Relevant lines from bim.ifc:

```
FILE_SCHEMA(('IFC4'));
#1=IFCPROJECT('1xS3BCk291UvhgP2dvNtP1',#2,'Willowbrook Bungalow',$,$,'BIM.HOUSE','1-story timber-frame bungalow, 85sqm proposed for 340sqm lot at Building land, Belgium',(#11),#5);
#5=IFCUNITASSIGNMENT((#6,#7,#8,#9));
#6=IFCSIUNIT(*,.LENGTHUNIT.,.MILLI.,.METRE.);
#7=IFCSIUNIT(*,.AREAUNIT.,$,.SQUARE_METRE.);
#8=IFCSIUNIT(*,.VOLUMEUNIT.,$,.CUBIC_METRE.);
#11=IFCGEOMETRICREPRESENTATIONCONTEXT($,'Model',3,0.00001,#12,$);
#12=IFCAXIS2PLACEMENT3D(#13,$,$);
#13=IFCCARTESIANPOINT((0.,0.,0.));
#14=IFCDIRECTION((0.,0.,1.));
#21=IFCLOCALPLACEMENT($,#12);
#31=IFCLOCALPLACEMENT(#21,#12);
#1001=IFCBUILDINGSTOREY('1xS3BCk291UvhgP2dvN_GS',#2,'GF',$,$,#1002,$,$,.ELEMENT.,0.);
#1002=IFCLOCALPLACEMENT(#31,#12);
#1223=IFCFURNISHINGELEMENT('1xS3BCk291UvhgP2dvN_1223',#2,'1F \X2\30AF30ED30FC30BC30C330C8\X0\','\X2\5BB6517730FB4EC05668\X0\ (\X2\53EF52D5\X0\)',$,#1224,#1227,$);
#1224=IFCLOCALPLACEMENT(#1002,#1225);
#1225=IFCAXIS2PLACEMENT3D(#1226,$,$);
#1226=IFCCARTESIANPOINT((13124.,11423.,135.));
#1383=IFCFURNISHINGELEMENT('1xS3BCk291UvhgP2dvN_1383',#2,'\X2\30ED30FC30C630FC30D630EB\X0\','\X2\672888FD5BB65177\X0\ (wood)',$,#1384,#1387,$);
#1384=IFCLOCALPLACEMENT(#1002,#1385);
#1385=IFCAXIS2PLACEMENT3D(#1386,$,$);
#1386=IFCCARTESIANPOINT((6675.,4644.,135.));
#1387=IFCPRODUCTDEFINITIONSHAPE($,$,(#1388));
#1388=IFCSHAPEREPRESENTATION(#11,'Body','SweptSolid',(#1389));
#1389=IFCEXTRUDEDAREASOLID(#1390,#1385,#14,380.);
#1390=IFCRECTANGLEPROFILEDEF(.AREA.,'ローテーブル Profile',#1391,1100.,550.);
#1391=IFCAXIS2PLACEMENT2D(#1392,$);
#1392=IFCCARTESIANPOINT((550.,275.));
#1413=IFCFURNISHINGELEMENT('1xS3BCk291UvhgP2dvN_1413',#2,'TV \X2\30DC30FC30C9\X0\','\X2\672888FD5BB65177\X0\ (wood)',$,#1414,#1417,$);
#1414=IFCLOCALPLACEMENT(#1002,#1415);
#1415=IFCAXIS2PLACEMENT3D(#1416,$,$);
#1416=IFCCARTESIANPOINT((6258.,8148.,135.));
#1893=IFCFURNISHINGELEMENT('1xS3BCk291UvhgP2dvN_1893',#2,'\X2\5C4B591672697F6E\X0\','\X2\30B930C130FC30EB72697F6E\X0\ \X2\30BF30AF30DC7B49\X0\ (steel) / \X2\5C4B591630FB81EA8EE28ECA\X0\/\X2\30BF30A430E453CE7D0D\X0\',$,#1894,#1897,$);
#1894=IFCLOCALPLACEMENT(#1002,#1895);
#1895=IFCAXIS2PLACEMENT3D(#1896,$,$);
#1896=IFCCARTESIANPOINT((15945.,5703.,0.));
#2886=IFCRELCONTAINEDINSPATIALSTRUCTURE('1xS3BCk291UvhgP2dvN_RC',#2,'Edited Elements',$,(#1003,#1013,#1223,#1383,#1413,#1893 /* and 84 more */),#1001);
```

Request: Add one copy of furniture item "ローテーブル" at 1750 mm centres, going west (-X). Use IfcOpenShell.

```python
import numpy as np
import ifcopenshell
import ifcopenshell.api.geometry
import ifcopenshell.api.root
import ifcopenshell.util.element
import ifcopenshell.util.placement
import ifcopenshell.util.unit

model = ifcopenshell.open("bim.ifc")
unit_scale = ifcopenshell.util.unit.calculate_unit_scale(model)


def reuse_history(source, copy):
    """copy_class also copies each property set's owner history, people and application; keep the originals."""
    for rel in copy.IsDefinedBy:
        if rel.is_a("IfcRelDefinesByProperties") and (history := rel.RelatingPropertyDefinition.OwnerHistory):
            rel.RelatingPropertyDefinition.OwnerHistory = source.OwnerHistory
            ifcopenshell.util.element.remove_deep2(model, history)


source = model.by_id(1383)
base = ifcopenshell.util.placement.get_local_placement(source.ObjectPlacement)
step = np.array([-1.0, 0.0, 0.0]) * 1.75 / unit_scale

for i in range(1, 2):
    copy = ifcopenshell.api.root.copy_class(model, product=source)
    copy.Representation = ifcopenshell.util.element.copy_deep(
        model, source.Representation, exclude=["IfcGeometricRepresentationContext", "IfcRepresentationMap"]
    )
    reuse_history(source, copy)
    matrix = base.copy()
    matrix[:3, 3] += i * step
    print("added at", matrix[:3, 3].round(3) + 0.0)
    ifcopenshell.api.geometry.edit_object_placement(model, product=copy, matrix=matrix, is_si=False)

model.write("bim_v2.ifc")
```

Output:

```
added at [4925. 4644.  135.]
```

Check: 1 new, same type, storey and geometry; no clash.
